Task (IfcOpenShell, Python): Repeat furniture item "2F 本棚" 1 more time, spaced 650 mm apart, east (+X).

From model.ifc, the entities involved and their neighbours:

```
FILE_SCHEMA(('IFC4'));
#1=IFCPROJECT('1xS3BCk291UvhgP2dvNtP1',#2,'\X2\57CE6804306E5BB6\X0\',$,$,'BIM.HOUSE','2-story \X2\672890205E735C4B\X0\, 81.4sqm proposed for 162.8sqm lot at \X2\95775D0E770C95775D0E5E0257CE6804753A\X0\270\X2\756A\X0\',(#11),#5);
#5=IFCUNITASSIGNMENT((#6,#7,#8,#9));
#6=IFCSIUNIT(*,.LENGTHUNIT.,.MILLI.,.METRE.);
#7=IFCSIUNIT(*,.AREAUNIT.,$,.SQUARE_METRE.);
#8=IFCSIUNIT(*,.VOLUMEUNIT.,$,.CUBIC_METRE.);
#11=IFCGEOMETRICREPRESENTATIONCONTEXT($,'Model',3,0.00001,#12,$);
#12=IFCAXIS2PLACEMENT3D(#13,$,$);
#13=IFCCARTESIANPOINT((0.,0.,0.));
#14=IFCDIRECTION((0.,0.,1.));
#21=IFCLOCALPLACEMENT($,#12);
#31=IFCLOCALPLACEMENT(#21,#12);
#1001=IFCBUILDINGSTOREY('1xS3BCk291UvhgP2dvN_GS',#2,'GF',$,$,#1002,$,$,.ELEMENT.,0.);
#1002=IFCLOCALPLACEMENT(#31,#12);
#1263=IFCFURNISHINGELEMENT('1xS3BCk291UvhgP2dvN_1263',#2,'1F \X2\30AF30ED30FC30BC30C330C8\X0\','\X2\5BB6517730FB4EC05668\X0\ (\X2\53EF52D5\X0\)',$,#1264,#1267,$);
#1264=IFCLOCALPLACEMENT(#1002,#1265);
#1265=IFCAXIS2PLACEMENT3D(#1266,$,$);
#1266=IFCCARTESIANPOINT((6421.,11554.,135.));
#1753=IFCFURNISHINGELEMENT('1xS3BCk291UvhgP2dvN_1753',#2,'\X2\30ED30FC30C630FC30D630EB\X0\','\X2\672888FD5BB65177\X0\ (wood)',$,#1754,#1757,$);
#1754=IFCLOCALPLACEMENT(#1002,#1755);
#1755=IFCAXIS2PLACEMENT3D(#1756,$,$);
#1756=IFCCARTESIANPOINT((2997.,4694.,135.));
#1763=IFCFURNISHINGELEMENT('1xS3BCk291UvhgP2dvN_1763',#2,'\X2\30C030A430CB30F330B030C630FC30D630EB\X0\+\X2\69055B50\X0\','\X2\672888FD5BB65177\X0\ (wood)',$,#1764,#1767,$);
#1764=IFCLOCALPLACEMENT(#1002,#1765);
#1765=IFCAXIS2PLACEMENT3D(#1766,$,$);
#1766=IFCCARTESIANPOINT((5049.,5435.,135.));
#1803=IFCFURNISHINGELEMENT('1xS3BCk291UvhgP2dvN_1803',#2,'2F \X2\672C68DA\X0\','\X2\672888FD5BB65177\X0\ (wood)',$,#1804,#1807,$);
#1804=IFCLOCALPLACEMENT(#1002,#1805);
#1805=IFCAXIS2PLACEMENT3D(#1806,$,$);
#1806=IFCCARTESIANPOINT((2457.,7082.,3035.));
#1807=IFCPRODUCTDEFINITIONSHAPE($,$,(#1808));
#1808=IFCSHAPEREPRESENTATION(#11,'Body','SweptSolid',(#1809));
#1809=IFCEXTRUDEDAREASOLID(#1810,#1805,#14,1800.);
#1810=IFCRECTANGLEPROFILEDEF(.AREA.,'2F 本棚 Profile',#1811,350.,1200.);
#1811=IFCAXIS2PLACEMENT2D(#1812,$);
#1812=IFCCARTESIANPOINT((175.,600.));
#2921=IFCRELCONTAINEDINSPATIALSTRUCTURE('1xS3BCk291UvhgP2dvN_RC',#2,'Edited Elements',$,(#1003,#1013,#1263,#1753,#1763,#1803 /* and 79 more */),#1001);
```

```python
import numpy as np
import ifcopenshell
import ifcopenshell.api.geometry
import ifcopenshell.api.root
import ifcopenshell.util.element
import ifcopenshell.util.placement
import ifcopenshell.util.unit

model = ifcopenshell.open("model.ifc")
unit_scale = ifcopenshell.util.unit.calculate_unit_scale(model)


def reuse_history(source, copy):
    """copy_class also copies each property set's owner history, people and application; keep the originals."""
    for rel in copy.IsDefinedBy:
        if rel.is_a("IfcRelDefinesByProperties") and (history := rel.RelatingPropertyDefinition.OwnerHistory):
            rel.RelatingPropertyDefinition.OwnerHistory = source.OwnerHistory
            ifcopenshell.util.element.remove_deep2(model, history)


source = model.by_guid("1xS3BCk291UvhgP2dvN_1803")
base = ifcopenshell.util.placement.get_local_placement(source.ObjectPlacement)
step = np.array([1.0, 0.0, 0.0]) * 0.65 / unit_scale

for i in range(1, 2):
    copy = ifcopenshell.api.root.copy_class(model, product=source)
    copy.Representation = ifcopenshell.util.element.copy_deep(
        model, source.Representation, exclude=["IfcGeometricRepresentationContext", "IfcRepresentationMap"]
    )
    reuse_history(source, copy)
    matrix = base.copy()
    matrix[:3, 3] += i * step
    print("added at", matrix[:3, 3].round(3) + 0.0)
    ifcopenshell.api.geometry.edit_object_placement(model, product=copy, matrix=matrix, is_si=False)

model.write("model_v2.ifc")
```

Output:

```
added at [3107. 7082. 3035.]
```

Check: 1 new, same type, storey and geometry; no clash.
